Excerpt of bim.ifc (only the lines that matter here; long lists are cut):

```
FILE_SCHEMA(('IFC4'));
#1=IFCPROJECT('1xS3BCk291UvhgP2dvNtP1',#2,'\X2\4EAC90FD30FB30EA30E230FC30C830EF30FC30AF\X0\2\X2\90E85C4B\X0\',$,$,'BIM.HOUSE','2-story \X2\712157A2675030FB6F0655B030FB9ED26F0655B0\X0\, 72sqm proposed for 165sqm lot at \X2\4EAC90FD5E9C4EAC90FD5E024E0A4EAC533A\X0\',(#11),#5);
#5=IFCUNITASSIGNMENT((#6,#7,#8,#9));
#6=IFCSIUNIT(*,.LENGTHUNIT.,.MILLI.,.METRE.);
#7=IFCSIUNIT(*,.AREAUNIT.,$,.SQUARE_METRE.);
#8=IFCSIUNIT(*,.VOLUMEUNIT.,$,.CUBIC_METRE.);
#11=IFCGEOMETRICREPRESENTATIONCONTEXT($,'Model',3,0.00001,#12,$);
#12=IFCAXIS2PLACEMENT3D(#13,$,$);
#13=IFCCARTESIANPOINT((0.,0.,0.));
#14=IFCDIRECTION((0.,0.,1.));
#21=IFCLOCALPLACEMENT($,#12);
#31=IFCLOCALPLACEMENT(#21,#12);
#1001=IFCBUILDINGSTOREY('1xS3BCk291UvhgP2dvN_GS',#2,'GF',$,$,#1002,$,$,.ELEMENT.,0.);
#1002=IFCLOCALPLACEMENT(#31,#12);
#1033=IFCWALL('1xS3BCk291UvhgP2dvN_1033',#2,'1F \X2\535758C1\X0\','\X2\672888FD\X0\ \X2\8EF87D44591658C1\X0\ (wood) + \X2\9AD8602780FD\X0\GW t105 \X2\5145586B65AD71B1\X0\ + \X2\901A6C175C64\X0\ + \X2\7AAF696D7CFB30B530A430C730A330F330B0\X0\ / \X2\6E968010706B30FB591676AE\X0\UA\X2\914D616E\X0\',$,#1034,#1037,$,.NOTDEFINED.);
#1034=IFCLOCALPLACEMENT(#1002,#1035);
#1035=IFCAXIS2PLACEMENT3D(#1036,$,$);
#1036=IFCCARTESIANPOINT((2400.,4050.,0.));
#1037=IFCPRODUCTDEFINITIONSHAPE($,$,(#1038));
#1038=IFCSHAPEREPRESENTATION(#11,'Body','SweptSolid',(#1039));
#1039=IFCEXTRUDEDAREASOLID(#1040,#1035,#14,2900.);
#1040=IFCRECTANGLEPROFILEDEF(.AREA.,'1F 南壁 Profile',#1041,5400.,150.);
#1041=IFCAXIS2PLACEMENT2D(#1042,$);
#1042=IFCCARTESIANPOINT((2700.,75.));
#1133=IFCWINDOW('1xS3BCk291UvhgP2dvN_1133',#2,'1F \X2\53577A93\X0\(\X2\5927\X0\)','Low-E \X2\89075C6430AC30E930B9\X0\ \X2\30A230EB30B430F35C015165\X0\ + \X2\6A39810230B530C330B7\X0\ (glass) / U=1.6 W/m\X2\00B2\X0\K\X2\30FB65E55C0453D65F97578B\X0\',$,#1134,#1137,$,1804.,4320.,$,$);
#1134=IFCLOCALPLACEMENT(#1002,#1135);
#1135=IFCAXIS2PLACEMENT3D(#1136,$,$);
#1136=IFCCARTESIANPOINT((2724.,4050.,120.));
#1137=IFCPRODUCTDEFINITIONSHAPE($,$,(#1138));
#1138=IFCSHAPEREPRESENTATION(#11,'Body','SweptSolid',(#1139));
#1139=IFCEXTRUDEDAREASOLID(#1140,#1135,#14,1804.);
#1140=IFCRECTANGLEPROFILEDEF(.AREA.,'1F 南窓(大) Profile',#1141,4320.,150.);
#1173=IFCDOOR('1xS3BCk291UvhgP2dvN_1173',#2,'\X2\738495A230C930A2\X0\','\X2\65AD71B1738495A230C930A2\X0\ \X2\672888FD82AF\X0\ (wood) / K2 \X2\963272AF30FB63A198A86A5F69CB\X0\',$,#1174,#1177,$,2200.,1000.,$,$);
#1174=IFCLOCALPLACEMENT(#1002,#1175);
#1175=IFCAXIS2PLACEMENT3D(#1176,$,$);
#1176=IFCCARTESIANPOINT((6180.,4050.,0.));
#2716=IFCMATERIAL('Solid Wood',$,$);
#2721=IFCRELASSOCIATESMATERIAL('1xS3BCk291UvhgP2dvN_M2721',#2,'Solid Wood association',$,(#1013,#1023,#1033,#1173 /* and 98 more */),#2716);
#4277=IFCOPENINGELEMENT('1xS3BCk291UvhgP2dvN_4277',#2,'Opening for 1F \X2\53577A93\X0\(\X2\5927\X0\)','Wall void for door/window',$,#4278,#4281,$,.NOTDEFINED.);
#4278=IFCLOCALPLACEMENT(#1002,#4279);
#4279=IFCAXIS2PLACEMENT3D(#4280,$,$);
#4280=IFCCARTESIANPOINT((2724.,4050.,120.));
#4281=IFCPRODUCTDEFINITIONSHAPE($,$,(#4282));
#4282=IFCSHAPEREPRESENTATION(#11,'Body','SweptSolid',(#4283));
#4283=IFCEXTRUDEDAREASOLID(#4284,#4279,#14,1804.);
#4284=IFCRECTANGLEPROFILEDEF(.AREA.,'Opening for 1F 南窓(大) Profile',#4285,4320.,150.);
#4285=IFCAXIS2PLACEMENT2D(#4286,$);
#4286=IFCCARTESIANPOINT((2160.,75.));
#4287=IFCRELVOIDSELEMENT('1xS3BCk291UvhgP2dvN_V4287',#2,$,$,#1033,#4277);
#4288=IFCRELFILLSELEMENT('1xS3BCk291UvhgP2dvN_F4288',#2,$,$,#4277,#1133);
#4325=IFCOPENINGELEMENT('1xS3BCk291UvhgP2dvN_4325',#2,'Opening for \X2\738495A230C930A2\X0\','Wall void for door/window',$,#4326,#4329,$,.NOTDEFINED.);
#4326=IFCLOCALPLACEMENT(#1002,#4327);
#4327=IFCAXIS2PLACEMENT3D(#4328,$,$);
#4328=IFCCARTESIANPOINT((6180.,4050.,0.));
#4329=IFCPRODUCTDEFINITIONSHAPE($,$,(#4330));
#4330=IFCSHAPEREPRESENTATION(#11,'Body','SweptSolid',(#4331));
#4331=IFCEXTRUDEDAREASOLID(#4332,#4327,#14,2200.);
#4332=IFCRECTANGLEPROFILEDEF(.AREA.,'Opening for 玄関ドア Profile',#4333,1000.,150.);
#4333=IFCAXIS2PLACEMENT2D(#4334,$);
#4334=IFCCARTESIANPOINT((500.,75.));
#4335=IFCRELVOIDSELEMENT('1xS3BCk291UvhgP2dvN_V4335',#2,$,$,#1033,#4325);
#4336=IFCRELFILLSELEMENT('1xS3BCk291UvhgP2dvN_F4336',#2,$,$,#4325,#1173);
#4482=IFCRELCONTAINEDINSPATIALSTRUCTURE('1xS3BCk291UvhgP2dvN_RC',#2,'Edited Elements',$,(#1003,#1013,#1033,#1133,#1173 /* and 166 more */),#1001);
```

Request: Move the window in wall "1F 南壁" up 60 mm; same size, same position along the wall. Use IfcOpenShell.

```python
import numpy as np
import ifcopenshell
import ifcopenshell.api.geometry
import ifcopenshell.util.placement
import ifcopenshell.util.unit

model = ifcopenshell.open("bim.ifc")
unit_scale = ifcopenshell.util.unit.calculate_unit_scale(model)

window = model.by_id(1133)
opening = window.FillsVoids[0].RelatingOpeningElement
dz = 0.06 / unit_scale

shift = np.array([0.0, 0.0, dz])
# The window is not placed relative to its opening, so move both.
for product in (opening, window):
    matrix = ifcopenshell.util.placement.get_local_placement(product.ObjectPlacement)
    matrix[:3, 3] += shift
    ifcopenshell.api.geometry.edit_object_placement(model, product=product, matrix=matrix, is_si=False)

print(f"moved by {dz * unit_scale:+.3f} m")

model.write("bim-out.ifc")
```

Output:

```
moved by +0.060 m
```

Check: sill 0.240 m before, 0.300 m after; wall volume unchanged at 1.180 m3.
